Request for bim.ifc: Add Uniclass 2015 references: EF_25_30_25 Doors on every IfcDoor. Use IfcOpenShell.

First a look at what the model holds.

```python
import ifcopenshell

model = ifcopenshell.open("bim.ifc")
print(model.schema)
print("classifications:", [c.Name for c in model.by_type("IfcClassification")])
for ifc_class in ("IfcDoor", "IfcRoof", "IfcStair", "IfcWall", "IfcWindow"):
    print(ifc_class, len(model.by_type(ifc_class)))
```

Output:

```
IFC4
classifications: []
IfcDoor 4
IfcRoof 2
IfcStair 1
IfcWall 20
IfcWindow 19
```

```python
import ifcopenshell
import ifcopenshell.api.classification

model = ifcopenshell.open("bim.ifc")

system = ifcopenshell.api.classification.add_classification(model, classification="Uniclass 2015")

codes = {
    "IfcDoor": ("EF_25_30_25", "Doors"),
}
for ifc_class, (code, name) in codes.items():
    products = model.by_type(ifc_class)
    ifcopenshell.api.classification.add_reference(
        model, products=products, classification=system, identification=code, name=name
    )
    print(code, len(products))

model.write("bim_v2.ifc")
```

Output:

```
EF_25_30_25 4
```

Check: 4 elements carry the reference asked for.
